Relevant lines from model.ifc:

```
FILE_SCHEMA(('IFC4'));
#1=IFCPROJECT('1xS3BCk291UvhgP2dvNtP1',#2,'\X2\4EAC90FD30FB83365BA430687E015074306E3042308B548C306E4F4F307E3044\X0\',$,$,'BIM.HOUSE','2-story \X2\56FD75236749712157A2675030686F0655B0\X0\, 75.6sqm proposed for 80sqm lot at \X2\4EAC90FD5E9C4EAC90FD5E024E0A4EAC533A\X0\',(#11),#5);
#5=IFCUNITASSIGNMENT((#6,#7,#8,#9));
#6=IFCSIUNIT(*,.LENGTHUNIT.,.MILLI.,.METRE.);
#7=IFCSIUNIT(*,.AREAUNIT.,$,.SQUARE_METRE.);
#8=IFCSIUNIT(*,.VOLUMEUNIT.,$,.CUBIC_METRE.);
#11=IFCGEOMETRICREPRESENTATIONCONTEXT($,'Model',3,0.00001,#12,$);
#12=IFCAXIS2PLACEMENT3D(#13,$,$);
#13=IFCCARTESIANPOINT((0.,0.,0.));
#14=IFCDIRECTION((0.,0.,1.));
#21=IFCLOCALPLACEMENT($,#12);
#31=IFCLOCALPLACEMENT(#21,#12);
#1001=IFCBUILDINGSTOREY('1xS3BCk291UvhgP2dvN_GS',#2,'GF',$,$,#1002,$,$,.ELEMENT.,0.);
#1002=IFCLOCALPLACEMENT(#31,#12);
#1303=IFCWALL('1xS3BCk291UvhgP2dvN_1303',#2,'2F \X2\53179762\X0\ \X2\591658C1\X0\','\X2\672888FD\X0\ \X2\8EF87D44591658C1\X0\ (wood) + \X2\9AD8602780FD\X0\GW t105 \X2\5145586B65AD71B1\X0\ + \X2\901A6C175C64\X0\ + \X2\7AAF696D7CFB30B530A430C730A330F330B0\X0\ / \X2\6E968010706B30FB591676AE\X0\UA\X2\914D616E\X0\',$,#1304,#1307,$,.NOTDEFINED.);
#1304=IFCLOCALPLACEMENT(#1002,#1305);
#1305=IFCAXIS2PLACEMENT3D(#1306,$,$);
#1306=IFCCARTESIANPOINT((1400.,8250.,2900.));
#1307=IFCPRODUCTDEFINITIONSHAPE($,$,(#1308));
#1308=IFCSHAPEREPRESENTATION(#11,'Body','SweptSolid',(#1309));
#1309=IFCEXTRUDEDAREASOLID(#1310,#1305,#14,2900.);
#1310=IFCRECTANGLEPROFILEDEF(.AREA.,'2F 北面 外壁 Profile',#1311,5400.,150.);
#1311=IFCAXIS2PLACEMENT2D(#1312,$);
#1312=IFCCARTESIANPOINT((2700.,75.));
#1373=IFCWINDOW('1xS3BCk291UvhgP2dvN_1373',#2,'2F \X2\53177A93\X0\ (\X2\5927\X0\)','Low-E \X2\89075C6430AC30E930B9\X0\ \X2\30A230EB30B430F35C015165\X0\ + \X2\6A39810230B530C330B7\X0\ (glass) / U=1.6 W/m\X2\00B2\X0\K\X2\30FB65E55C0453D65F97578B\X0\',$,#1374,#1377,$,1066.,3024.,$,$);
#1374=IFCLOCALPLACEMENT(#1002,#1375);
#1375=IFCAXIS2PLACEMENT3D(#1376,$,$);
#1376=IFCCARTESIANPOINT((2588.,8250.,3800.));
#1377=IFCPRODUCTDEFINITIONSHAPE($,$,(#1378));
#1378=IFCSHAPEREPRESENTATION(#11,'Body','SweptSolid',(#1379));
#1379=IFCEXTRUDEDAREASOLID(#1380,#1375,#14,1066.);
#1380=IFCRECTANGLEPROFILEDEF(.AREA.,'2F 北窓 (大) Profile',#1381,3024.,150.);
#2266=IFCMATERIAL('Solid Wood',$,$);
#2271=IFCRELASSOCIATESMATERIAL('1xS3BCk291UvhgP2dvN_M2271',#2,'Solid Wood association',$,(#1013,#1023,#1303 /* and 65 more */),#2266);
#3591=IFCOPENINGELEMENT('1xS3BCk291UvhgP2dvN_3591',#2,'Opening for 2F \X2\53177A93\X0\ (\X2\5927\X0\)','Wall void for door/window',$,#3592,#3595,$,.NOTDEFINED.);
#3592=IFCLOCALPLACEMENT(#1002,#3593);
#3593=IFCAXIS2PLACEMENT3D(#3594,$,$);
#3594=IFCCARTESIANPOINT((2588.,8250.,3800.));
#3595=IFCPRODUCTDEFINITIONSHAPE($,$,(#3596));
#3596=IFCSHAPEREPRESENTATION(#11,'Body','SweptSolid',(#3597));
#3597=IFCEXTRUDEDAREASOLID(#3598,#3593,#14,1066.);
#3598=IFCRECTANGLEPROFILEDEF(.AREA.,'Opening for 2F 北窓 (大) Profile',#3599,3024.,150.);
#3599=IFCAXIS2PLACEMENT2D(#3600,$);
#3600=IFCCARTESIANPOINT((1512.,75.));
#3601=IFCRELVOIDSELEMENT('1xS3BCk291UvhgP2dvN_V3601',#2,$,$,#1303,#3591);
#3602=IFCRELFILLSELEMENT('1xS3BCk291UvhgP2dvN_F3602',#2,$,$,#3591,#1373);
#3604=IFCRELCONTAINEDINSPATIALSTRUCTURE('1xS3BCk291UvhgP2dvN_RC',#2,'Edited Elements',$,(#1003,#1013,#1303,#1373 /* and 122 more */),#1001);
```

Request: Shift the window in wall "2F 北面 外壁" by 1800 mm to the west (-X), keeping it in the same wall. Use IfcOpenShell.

```python
import ifcopenshell
import ifcopenshell.api.geometry
import ifcopenshell.util.placement

model = ifcopenshell.open("model.ifc")

window = model.by_guid("1xS3BCk291UvhgP2dvN_1373")
opening = window.FillsVoids[0].RelatingOpeningElement
wall = opening.VoidsElements[0].RelatingBuildingElement

wall_matrix = ifcopenshell.util.placement.get_local_placement(wall.ObjectPlacement)
shift = wall_matrix[:3, 0] * -1800.0
before = ifcopenshell.util.placement.get_local_placement(window.ObjectPlacement)[:3, 3].copy()

# The window is not placed relative to its opening, so move both.
for product in (opening, window):
    matrix = ifcopenshell.util.placement.get_local_placement(product.ObjectPlacement)
    matrix[:3, 3] += shift
    ifcopenshell.api.geometry.edit_object_placement(model, product=product, matrix=matrix, is_si=False)

after = ifcopenshell.util.placement.get_local_placement(window.ObjectPlacement)[:3, 3]
print("window moved by", (after - before).round(3) + 0.0)

model.write("model_rev.ifc")
```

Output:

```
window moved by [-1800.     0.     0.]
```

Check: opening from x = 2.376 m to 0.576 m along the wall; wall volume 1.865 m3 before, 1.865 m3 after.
